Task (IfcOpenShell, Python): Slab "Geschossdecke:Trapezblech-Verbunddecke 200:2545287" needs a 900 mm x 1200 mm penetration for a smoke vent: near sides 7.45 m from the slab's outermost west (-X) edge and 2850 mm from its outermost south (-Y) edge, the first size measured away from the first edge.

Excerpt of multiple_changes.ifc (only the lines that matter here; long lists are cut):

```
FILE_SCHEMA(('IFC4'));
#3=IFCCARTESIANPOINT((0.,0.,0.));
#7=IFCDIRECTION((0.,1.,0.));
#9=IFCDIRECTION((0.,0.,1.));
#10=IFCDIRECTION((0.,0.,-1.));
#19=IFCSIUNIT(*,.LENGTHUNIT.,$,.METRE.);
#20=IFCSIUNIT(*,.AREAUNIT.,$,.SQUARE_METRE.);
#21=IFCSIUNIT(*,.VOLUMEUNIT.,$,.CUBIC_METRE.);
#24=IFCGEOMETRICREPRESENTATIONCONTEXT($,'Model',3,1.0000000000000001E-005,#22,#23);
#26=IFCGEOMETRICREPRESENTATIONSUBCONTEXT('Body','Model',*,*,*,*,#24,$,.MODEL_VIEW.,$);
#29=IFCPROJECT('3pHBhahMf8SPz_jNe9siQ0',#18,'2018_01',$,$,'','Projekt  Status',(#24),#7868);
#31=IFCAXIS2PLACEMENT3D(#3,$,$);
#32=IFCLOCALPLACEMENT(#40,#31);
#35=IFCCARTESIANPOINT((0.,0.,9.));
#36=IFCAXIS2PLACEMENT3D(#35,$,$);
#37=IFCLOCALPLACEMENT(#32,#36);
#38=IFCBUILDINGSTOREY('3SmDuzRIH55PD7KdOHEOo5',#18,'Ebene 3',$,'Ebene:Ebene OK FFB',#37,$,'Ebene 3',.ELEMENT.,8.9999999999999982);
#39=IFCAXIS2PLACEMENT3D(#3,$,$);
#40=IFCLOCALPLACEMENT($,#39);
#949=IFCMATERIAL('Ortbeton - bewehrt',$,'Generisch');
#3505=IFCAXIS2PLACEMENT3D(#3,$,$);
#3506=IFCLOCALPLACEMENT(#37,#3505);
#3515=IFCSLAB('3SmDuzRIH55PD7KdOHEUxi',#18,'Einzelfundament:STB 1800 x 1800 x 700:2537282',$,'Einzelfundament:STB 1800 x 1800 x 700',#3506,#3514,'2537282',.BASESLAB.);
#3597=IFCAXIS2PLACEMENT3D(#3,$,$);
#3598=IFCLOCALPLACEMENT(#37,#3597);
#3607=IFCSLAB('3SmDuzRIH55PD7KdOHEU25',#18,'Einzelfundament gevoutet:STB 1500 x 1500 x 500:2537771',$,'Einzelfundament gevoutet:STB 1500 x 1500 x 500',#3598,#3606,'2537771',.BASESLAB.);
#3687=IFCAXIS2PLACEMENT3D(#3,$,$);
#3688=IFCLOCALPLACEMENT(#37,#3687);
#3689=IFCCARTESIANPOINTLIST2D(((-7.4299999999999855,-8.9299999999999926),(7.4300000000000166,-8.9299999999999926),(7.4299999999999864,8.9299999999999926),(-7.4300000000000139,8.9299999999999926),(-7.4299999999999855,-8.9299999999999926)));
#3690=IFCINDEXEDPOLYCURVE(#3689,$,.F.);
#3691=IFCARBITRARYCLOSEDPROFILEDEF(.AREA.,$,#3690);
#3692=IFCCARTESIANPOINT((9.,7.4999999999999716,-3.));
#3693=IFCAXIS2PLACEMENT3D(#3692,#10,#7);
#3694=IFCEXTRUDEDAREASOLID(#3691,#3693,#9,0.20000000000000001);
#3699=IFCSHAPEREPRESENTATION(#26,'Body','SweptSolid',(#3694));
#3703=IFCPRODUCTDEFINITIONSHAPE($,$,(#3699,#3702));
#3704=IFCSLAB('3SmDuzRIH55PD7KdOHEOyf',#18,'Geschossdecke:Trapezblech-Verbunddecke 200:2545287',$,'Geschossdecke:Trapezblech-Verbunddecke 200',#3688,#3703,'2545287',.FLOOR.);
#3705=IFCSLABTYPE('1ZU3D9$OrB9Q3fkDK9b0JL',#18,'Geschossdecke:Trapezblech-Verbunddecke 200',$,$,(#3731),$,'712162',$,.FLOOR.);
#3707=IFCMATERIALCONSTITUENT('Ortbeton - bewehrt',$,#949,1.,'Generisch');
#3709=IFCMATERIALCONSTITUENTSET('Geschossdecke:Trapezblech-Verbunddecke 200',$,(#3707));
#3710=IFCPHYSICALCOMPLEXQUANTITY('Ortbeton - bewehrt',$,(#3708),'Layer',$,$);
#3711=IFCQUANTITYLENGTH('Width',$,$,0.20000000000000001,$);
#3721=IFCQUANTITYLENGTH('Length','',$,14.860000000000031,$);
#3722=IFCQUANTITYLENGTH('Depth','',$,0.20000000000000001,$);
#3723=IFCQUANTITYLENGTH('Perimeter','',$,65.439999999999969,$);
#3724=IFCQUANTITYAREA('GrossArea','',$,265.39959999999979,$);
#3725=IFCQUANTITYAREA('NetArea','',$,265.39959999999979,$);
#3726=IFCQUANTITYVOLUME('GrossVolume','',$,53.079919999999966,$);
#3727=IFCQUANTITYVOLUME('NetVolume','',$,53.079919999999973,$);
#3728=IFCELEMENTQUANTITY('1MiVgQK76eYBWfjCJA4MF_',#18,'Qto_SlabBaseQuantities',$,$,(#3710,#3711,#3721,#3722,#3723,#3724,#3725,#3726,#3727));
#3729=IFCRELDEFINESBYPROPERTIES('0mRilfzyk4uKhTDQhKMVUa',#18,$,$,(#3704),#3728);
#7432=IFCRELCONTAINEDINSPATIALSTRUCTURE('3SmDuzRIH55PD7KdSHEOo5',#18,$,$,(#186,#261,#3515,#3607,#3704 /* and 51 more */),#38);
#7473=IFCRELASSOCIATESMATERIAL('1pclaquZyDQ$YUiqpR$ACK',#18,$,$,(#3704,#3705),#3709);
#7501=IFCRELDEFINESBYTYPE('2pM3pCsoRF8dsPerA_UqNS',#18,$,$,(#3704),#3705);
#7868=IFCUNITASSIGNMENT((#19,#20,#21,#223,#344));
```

```python
import numpy as np
import ifcopenshell
import ifcopenshell.api.feature
import ifcopenshell.api.geometry
import ifcopenshell.api.pset
import ifcopenshell.api.root
import ifcopenshell.geom
import ifcopenshell.util.element
import ifcopenshell.util.placement
import ifcopenshell.util.representation
import ifcopenshell.util.shape
import ifcopenshell.util.unit

model = ifcopenshell.open("multiple_changes.ifc")
unit_scale = ifcopenshell.util.unit.calculate_unit_scale(model)
area_scale = ifcopenshell.util.unit.calculate_unit_scale(model, "AREAUNIT")
volume_scale = ifcopenshell.util.unit.calculate_unit_scale(model, "VOLUMEUNIT")
settings = ifcopenshell.geom.settings()


def volume(element):
    """Net volume in cubic metres, openings subtracted."""
    shape = ifcopenshell.geom.create_shape(settings, element)
    return ifcopenshell.util.shape.get_volume(shape.geometry)


slab = model.by_id(3704)
before = volume(slab)

# Extent in the slab's own axes, in metres. The edges named are its -X and -Y sides.
slab_shape = ifcopenshell.geom.create_shape(settings, slab)
vertices = ifcopenshell.util.shape.get_vertices(slab_shape.geometry)
x_min, y_min, bottom = vertices.min(axis=0)
top = vertices[:, 2].max()

opening = ifcopenshell.api.root.create_entity(model, ifc_class="IfcOpeningElement", name="Smoke vent opening", predefined_type="OPENING")
context = ifcopenshell.util.representation.get_context(model, "Model", "Body", "MODEL_VIEW")
width, depth = 0.9, 1.2
outline = [(0.0, 0.0), (width, 0.0), (width, depth), (0.0, depth), (0.0, 0.0)]
# Overshoot both faces by 50 mm so the cut is clean.
shape = ifcopenshell.api.geometry.add_slab_representation(
    model, context=context, depth=top - bottom + 0.1, polyline=outline
)
ifcopenshell.api.geometry.assign_representation(model, product=opening, representation=shape)

matrix = ifcopenshell.util.placement.get_local_placement(slab.ObjectPlacement)
matrix[:, 3] = matrix @ np.append(np.array([x_min + 7.45, y_min + 2.85, bottom - 0.05]) / unit_scale, 1.0)
ifcopenshell.api.geometry.edit_object_placement(model, product=opening, matrix=matrix, is_si=False)
ifcopenshell.api.feature.add_feature(model, feature=opening, element=slab)

after = volume(slab)

# Update the slab's stored quantities.
qto = model.by_id(ifcopenshell.util.element.get_pset(slab, "Qto_SlabBaseQuantities", should_inherit=False)["id"])
ifcopenshell.api.pset.edit_qto(model, qto=qto, properties={
    "NetArea": after / (top - bottom) / area_scale,
    "NetVolume": after / volume_scale,
})

print(f"slab volume {before:.3f} -> {after:.3f} m3")

model.write("multiple_changes_rev.ifc")
```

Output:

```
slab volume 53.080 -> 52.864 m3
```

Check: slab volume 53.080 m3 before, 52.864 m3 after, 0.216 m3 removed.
